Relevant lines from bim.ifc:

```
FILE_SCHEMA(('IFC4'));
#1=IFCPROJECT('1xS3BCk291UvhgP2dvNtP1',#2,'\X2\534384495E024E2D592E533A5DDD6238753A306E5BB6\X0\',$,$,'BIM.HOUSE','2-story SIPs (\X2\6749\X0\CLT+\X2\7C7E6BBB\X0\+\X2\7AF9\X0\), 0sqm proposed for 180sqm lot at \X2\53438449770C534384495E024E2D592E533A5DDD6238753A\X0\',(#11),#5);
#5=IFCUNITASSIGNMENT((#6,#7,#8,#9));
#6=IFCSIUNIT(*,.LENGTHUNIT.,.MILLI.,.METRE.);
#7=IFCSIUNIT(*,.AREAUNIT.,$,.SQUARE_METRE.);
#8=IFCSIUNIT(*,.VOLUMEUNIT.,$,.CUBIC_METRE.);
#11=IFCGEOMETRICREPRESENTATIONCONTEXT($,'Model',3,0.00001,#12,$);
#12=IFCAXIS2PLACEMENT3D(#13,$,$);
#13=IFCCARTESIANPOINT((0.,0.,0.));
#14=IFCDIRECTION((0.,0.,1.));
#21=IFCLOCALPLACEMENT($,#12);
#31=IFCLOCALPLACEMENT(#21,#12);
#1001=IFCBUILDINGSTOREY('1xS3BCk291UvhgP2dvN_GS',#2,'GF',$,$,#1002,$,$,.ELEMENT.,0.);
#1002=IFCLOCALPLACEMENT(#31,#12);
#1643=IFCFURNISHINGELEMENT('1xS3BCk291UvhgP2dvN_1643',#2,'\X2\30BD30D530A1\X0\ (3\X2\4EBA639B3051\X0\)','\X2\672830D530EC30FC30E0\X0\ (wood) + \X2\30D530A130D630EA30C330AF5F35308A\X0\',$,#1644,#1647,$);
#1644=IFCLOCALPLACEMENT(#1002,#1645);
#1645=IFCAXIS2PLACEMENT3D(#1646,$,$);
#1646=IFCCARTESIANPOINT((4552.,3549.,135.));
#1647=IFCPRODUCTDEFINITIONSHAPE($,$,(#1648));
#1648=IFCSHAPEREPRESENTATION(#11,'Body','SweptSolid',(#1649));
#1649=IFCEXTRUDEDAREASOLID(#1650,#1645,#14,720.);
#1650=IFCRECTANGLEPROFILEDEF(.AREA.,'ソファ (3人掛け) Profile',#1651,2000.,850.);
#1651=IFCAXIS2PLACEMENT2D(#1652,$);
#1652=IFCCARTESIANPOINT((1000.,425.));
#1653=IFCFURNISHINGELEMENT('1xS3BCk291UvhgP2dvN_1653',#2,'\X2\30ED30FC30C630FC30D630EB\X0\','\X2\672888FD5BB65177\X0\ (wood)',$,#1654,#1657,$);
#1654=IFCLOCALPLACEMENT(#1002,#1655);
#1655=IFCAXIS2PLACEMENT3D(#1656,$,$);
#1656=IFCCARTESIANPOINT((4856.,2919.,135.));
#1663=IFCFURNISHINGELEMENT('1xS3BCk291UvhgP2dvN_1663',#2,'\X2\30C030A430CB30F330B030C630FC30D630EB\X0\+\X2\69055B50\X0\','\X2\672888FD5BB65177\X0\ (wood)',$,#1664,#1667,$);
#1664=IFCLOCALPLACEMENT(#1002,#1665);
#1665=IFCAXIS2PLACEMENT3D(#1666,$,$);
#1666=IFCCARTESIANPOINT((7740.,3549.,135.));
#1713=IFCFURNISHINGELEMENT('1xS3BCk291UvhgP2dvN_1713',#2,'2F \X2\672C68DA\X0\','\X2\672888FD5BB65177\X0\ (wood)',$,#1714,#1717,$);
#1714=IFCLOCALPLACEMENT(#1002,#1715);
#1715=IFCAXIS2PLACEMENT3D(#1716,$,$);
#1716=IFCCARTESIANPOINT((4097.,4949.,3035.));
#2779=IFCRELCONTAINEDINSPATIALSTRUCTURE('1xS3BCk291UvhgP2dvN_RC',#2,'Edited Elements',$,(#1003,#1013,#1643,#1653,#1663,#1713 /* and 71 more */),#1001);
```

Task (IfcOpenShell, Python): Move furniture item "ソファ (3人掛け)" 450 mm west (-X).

```python
import ifcopenshell
import ifcopenshell.api.geometry
import ifcopenshell.util.placement
import ifcopenshell.util.unit

model = ifcopenshell.open("bim.ifc")
unit_scale = ifcopenshell.util.unit.calculate_unit_scale(model)

item = model.by_guid("1xS3BCk291UvhgP2dvN_1643")
matrix = ifcopenshell.util.placement.get_local_placement(item.ObjectPlacement)
matrix[0, 3] -= 0.45 / unit_scale
ifcopenshell.api.geometry.edit_object_placement(model, product=item, matrix=matrix, is_si=False)

print(ifcopenshell.util.placement.get_local_placement(item.ObjectPlacement).round(3) + 0.0)

model.write("bim_rev.ifc")
```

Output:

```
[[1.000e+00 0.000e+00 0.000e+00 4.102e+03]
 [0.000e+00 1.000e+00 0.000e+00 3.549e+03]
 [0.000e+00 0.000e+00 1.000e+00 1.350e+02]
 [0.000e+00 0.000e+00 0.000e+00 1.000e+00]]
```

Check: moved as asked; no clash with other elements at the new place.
